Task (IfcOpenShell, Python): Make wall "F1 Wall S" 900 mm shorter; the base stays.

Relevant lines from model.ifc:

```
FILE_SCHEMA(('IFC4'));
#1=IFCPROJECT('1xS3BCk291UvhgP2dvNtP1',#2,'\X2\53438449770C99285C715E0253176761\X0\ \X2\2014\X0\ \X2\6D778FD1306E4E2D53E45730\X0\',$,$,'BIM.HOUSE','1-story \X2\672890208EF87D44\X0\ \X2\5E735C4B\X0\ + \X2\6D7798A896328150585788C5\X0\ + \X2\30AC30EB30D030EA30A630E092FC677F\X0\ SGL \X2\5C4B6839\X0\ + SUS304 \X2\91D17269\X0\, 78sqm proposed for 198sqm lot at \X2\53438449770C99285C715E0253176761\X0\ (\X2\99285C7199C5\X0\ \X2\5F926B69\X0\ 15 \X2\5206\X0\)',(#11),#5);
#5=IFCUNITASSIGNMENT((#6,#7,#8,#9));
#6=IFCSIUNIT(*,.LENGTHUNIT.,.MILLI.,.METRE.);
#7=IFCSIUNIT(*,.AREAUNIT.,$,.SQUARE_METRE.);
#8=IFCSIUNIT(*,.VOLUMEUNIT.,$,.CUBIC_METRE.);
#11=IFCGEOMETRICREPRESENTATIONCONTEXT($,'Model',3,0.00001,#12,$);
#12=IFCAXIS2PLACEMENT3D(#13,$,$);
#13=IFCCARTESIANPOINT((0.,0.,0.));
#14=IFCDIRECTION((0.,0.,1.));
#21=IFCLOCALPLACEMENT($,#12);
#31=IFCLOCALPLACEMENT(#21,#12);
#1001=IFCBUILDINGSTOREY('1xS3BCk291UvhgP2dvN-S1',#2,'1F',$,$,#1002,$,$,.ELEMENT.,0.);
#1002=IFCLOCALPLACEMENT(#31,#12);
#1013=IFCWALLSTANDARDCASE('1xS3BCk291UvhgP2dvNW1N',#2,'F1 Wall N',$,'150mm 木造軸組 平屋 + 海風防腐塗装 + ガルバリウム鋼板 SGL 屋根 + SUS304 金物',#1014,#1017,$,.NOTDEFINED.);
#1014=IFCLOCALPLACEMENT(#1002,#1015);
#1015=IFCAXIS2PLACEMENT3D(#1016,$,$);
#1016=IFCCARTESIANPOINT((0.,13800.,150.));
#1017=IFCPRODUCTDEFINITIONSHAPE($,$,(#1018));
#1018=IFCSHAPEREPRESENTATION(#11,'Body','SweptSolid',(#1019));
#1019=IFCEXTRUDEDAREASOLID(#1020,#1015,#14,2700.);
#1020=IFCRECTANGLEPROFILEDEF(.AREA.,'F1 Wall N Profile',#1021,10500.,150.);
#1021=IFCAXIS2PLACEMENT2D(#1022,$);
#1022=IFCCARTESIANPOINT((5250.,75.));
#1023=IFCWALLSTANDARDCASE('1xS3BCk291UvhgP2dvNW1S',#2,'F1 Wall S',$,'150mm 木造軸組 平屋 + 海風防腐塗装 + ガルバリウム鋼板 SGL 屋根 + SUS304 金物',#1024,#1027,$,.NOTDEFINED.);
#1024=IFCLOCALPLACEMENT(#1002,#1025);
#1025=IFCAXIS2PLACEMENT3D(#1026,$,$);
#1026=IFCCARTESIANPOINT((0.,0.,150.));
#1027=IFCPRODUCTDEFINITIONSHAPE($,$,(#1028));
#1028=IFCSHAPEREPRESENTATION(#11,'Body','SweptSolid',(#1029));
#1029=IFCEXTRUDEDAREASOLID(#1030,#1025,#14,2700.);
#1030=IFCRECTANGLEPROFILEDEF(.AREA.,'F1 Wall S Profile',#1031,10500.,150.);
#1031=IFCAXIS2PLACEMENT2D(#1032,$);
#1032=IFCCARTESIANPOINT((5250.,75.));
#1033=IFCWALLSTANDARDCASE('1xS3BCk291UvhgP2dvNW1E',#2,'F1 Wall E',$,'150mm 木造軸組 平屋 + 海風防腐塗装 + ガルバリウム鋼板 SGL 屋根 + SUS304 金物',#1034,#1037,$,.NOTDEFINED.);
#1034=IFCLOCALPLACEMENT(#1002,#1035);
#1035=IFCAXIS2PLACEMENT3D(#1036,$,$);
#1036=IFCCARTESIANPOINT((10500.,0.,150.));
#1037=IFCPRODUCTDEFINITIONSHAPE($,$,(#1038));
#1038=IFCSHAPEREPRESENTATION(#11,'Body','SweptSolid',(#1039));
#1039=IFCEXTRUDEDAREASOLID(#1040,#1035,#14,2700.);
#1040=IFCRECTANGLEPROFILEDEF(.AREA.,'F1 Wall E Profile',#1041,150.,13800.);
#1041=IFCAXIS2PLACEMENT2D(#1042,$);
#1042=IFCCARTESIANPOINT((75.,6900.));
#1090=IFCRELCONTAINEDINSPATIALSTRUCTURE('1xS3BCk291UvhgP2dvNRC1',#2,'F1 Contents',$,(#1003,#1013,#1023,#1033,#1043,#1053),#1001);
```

```python
import ifcopenshell
import ifcopenshell.geom
import ifcopenshell.util.shape
import ifcopenshell.util.unit

model = ifcopenshell.open("model.ifc")
unit_scale = ifcopenshell.util.unit.calculate_unit_scale(model)
settings = ifcopenshell.geom.settings()


def volume(element):
    """Net volume in cubic metres, openings subtracted."""
    shape = ifcopenshell.geom.create_shape(settings, element)
    return ifcopenshell.util.shape.get_volume(shape.geometry)


wall = model.by_id(1023)
before = volume(wall)

body = next(r for r in wall.Representation.Representations if r.RepresentationIdentifier == "Body")
solid = body.Items[0]
old_height = solid.Depth
solid.Depth -= 0.9 / unit_scale
after = volume(wall)

print(f"height {old_height:g} -> {solid.Depth:g}, volume {before:.3f} -> {after:.3f} m3")

model.write("model-out.ifc")
```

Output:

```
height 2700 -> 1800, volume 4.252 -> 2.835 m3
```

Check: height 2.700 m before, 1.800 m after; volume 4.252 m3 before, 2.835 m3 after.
